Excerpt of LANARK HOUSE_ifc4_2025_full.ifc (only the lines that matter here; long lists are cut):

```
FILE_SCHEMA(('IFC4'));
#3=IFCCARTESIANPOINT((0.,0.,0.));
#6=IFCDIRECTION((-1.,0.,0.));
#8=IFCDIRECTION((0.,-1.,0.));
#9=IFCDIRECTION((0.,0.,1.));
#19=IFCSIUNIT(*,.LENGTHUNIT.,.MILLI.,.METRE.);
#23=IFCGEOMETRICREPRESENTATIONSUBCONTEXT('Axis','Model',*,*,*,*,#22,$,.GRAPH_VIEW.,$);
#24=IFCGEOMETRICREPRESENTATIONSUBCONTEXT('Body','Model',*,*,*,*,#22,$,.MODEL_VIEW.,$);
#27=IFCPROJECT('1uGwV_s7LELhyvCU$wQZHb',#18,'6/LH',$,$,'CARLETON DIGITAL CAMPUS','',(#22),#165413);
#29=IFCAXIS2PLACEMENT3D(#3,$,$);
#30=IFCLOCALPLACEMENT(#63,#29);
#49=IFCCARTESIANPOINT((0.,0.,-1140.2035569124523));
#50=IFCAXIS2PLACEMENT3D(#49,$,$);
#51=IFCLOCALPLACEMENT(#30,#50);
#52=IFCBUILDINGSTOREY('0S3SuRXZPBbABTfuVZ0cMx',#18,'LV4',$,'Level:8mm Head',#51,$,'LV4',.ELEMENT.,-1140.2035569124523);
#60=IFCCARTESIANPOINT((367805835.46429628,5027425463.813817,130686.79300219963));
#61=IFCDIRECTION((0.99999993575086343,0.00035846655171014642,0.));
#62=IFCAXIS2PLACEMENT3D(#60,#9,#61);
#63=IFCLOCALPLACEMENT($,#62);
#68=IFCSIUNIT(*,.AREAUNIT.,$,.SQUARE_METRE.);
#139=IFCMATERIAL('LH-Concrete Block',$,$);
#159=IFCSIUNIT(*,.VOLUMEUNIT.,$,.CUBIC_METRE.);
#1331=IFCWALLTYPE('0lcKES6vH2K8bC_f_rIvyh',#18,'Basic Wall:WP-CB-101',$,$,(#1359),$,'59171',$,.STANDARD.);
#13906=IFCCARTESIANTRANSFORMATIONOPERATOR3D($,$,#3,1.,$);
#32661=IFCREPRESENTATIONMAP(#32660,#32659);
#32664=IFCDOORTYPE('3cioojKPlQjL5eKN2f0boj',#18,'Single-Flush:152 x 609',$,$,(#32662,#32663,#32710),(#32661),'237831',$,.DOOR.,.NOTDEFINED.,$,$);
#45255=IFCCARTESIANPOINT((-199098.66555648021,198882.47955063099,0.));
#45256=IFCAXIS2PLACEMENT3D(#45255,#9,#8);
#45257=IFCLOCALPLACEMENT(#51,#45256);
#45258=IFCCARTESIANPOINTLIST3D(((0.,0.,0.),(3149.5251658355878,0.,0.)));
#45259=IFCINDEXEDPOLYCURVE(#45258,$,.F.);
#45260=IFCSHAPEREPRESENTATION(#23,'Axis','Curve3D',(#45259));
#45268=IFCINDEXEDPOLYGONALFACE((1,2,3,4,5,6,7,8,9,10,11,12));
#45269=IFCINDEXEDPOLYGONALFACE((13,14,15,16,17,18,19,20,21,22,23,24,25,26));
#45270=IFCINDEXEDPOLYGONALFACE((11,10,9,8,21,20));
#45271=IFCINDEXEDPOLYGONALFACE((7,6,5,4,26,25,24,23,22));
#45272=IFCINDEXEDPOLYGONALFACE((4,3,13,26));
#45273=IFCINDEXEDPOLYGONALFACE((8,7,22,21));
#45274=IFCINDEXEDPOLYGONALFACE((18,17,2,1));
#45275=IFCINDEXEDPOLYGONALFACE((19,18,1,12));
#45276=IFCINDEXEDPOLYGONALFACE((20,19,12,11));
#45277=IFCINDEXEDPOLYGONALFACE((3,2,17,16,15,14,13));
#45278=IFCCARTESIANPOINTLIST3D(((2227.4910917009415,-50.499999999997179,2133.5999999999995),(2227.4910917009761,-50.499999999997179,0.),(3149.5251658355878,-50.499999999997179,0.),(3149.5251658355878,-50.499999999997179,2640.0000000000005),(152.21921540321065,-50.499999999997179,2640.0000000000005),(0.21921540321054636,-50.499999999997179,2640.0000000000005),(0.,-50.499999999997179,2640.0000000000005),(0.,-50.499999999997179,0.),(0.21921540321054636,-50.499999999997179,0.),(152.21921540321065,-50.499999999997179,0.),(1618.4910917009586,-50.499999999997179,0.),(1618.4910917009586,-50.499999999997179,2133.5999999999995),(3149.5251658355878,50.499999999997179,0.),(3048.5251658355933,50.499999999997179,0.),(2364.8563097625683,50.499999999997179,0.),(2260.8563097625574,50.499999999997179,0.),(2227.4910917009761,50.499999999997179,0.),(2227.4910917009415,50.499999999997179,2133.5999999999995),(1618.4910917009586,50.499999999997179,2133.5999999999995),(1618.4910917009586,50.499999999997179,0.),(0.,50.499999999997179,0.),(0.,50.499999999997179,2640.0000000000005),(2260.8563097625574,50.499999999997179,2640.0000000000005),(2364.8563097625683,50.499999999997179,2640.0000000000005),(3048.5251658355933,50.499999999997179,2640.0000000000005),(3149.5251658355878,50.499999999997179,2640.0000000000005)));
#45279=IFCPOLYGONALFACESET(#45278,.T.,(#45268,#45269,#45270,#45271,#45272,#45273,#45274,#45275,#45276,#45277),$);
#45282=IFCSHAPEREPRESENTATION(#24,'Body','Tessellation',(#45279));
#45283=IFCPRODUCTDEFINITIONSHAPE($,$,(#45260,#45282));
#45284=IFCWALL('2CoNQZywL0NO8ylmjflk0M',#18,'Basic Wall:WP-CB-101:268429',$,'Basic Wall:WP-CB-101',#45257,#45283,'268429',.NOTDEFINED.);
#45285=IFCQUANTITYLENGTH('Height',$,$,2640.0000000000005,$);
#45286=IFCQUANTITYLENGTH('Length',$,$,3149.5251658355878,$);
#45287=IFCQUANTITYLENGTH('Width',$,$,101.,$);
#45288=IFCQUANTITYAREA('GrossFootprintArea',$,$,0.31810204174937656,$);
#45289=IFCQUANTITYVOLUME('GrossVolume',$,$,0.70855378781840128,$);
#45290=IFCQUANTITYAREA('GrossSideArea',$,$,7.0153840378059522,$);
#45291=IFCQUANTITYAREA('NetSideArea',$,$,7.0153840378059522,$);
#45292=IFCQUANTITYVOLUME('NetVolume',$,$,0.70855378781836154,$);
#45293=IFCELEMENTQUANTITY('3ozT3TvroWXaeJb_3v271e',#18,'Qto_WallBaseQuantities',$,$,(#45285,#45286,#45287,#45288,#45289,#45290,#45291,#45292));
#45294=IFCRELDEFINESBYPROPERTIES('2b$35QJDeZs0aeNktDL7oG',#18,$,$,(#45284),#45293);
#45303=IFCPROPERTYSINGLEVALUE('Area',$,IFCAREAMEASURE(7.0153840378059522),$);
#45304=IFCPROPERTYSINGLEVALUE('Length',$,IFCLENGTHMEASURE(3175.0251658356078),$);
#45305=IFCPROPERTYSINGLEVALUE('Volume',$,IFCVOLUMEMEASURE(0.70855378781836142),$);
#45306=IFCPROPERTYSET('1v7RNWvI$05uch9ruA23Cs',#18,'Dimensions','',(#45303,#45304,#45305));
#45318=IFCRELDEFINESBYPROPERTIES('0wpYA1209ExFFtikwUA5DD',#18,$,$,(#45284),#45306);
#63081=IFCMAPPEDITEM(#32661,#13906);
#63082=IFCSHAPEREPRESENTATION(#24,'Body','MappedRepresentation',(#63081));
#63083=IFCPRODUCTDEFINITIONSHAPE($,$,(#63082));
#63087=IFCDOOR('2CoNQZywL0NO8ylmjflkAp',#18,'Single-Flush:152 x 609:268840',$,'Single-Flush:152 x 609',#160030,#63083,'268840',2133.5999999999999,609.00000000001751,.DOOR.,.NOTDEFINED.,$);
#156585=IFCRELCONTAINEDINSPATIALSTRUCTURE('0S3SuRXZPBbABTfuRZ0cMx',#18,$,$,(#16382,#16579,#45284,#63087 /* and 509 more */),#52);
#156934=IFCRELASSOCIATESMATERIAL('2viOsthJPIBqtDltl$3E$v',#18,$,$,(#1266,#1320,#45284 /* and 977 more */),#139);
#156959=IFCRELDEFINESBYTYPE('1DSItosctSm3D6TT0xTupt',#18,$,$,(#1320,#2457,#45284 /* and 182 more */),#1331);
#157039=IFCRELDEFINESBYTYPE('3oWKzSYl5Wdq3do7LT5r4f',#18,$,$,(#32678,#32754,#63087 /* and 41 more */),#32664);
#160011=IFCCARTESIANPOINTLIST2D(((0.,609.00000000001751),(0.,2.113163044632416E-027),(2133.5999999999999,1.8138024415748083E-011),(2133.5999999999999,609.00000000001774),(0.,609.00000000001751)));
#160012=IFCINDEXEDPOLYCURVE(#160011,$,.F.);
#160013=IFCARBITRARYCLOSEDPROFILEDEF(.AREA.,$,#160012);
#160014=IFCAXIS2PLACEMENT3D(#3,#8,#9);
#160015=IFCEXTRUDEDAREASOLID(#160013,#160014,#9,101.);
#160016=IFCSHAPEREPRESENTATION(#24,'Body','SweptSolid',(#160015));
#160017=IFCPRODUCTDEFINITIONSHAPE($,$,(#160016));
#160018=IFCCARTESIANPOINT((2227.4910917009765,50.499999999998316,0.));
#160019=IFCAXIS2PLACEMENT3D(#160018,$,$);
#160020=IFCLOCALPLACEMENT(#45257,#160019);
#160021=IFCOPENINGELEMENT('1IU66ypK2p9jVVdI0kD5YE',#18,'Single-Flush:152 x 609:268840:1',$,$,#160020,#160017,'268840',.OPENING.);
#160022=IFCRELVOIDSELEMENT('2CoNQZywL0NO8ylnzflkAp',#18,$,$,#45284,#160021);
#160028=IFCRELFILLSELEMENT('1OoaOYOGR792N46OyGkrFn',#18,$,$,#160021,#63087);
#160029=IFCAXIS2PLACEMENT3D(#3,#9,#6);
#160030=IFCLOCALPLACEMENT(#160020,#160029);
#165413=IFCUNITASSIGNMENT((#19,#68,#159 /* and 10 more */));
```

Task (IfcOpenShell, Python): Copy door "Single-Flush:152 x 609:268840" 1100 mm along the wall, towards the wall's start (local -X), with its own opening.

```python
import ifcopenshell
import ifcopenshell.api.feature
import ifcopenshell.api.geometry
import ifcopenshell.api.pset
import ifcopenshell.api.root
import ifcopenshell.geom
import ifcopenshell.util.element
import ifcopenshell.util.placement
import ifcopenshell.util.shape
import ifcopenshell.util.unit

model = ifcopenshell.open("LANARK HOUSE_ifc4_2025_full.ifc")
area_scale = ifcopenshell.util.unit.calculate_unit_scale(model, "AREAUNIT")
volume_scale = ifcopenshell.util.unit.calculate_unit_scale(model, "VOLUMEUNIT")
settings = ifcopenshell.geom.settings()


def volume(element):
    """Net volume in cubic metres, openings subtracted."""
    shape = ifcopenshell.geom.create_shape(settings, element)
    return ifcopenshell.util.shape.get_volume(shape.geometry)


def reuse_history(source, copy):
    """copy_class also copies each property set's owner history, people and application; keep the originals."""
    for rel in copy.IsDefinedBy:
        if rel.is_a("IfcRelDefinesByProperties") and (history := rel.RelatingPropertyDefinition.OwnerHistory):
            rel.RelatingPropertyDefinition.OwnerHistory = source.OwnerHistory
            ifcopenshell.util.element.remove_deep2(model, history)


door = model.by_guid("2CoNQZywL0NO8ylmjflkAp")
opening = door.FillsVoids[0].RelatingOpeningElement
wall = opening.VoidsElements[0].RelatingBuildingElement
before = volume(wall)
shift = ifcopenshell.util.placement.get_local_placement(wall.ObjectPlacement)[:3, 0] * -1100.0

# copy_class copies the void relationship, type, container and properties, but no geometry.
new_opening = ifcopenshell.api.root.copy_class(model, product=opening)
new_opening.Representation = ifcopenshell.util.element.copy_deep(
    model, opening.Representation, exclude=["IfcGeometricRepresentationContext", "IfcRepresentationMap"]
)
new_opening.Name = "Single-Flush:152 x 609"
new_opening.Tag = None
reuse_history(opening, new_opening)
new_door = ifcopenshell.api.root.copy_class(model, product=door)
new_door.Representation = ifcopenshell.util.element.copy_deep(
    model, door.Representation, exclude=["IfcGeometricRepresentationContext", "IfcRepresentationMap"]
)
new_door.Name = "Single-Flush:152 x 609"
new_door.Tag = None
reuse_history(door, new_door)
ifcopenshell.api.feature.add_filling(model, opening=new_opening, element=new_door)

for old, new in ((opening, new_opening), (door, new_door)):
    matrix = ifcopenshell.util.placement.get_local_placement(old.ObjectPlacement)
    matrix[:3, 3] += shift
    ifcopenshell.api.geometry.edit_object_placement(model, product=new, matrix=matrix, is_si=False)

after = volume(wall)
thickness = 0.101  # wall thickness in metres

# Update the wall's stored quantities.
qto = model.by_id(ifcopenshell.util.element.get_pset(wall, "Qto_WallBaseQuantities", should_inherit=False)["id"])
ifcopenshell.api.pset.edit_qto(model, qto=qto, properties={
    "NetSideArea": after / thickness / area_scale,
    "NetVolume": after / volume_scale,
})
pset = model.by_id(ifcopenshell.util.element.get_pset(wall, "Dimensions", should_inherit=False)["id"])
ifcopenshell.api.pset.edit_pset(model, pset=pset, properties={
    "Area": model.create_entity("IfcAreaMeasure", after / thickness / area_scale),
    "Volume": model.create_entity("IfcVolumeMeasure", after / volume_scale),
})

print(f"wall volume {before:.3f} -> {after:.3f} m3")

model.write("LANARK HOUSE_ifc4_2025_full_v2.ifc")
```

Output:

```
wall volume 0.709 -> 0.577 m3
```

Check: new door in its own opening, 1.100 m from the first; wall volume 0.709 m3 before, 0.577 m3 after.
